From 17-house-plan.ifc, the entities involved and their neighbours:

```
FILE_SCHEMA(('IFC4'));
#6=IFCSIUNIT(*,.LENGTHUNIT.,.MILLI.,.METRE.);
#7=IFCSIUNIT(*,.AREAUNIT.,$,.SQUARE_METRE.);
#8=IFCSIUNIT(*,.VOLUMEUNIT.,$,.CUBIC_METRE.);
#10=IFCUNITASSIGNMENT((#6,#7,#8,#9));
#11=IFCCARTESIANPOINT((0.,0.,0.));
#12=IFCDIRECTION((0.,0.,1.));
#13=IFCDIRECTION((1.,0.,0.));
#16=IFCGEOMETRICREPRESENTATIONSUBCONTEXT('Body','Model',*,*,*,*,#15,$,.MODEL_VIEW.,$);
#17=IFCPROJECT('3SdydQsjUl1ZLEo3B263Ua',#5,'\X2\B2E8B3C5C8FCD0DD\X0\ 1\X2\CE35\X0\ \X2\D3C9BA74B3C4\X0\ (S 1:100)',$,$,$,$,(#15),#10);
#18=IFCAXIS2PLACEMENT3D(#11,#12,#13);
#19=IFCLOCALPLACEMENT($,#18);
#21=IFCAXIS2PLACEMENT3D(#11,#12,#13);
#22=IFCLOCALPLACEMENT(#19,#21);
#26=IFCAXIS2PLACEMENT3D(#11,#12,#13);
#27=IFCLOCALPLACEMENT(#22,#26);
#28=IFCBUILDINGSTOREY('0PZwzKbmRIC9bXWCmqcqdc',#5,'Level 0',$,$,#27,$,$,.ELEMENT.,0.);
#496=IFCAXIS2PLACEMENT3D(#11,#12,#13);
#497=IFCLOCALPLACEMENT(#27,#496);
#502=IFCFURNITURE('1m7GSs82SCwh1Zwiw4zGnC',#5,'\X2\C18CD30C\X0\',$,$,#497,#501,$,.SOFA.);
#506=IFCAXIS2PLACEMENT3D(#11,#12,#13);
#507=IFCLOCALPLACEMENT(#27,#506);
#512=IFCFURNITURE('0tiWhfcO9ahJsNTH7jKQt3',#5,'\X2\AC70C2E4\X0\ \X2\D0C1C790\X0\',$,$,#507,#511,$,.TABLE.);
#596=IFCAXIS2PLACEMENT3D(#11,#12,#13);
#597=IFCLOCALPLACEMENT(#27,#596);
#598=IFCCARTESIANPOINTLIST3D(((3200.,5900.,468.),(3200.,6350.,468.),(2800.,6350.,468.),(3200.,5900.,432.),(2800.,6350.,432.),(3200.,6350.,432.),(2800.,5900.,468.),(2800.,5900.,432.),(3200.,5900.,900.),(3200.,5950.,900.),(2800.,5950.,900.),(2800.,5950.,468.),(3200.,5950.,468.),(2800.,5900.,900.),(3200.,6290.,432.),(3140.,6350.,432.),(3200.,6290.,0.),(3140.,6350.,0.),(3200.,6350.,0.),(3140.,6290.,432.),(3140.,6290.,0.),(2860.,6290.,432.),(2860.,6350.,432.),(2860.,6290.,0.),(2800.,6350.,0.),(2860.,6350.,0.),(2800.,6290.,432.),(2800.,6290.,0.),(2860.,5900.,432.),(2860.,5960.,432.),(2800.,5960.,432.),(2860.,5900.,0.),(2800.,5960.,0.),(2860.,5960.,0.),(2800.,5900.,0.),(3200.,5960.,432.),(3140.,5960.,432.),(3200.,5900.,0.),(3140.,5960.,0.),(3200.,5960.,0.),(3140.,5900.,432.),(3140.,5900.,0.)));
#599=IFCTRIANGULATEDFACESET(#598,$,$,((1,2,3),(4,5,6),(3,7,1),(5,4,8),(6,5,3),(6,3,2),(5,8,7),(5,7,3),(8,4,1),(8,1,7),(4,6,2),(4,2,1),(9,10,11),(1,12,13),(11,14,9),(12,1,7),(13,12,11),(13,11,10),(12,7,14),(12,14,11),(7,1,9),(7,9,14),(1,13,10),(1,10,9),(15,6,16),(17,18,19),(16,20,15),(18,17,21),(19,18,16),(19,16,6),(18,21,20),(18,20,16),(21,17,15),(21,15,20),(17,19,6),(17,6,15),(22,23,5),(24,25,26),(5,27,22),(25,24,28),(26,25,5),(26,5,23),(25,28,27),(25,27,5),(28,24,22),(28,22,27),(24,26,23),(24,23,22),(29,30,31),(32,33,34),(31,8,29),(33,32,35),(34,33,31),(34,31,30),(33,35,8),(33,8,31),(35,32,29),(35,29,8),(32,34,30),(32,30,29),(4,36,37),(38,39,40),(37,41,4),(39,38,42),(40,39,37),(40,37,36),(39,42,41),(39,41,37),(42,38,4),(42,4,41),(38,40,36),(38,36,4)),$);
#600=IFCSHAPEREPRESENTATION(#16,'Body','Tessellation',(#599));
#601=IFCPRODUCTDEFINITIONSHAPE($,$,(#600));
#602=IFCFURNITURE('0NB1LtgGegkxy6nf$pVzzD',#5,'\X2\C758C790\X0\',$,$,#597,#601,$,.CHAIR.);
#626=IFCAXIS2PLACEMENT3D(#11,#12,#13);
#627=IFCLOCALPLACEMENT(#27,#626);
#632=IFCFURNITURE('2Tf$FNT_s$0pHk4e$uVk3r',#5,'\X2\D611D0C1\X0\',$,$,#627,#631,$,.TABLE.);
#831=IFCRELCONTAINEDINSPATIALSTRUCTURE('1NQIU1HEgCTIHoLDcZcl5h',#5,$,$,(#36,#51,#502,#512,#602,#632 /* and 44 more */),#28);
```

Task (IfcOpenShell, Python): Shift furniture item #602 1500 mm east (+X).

```python
import ifcopenshell
import ifcopenshell.api.geometry
import ifcopenshell.util.placement

model = ifcopenshell.open("17-house-plan.ifc")

item = model.by_id(602)
matrix = ifcopenshell.util.placement.get_local_placement(item.ObjectPlacement)
matrix[0, 3] += 1500.0
ifcopenshell.api.geometry.edit_object_placement(model, product=item, matrix=matrix, is_si=False)

print(ifcopenshell.util.placement.get_local_placement(item.ObjectPlacement).round(3) + 0.0)

model.write("17-house-plan_v2.ifc")
```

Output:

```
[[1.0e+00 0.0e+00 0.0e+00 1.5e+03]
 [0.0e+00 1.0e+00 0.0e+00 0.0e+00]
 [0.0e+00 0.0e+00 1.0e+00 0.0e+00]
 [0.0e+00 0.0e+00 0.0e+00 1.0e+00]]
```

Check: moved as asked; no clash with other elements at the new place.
